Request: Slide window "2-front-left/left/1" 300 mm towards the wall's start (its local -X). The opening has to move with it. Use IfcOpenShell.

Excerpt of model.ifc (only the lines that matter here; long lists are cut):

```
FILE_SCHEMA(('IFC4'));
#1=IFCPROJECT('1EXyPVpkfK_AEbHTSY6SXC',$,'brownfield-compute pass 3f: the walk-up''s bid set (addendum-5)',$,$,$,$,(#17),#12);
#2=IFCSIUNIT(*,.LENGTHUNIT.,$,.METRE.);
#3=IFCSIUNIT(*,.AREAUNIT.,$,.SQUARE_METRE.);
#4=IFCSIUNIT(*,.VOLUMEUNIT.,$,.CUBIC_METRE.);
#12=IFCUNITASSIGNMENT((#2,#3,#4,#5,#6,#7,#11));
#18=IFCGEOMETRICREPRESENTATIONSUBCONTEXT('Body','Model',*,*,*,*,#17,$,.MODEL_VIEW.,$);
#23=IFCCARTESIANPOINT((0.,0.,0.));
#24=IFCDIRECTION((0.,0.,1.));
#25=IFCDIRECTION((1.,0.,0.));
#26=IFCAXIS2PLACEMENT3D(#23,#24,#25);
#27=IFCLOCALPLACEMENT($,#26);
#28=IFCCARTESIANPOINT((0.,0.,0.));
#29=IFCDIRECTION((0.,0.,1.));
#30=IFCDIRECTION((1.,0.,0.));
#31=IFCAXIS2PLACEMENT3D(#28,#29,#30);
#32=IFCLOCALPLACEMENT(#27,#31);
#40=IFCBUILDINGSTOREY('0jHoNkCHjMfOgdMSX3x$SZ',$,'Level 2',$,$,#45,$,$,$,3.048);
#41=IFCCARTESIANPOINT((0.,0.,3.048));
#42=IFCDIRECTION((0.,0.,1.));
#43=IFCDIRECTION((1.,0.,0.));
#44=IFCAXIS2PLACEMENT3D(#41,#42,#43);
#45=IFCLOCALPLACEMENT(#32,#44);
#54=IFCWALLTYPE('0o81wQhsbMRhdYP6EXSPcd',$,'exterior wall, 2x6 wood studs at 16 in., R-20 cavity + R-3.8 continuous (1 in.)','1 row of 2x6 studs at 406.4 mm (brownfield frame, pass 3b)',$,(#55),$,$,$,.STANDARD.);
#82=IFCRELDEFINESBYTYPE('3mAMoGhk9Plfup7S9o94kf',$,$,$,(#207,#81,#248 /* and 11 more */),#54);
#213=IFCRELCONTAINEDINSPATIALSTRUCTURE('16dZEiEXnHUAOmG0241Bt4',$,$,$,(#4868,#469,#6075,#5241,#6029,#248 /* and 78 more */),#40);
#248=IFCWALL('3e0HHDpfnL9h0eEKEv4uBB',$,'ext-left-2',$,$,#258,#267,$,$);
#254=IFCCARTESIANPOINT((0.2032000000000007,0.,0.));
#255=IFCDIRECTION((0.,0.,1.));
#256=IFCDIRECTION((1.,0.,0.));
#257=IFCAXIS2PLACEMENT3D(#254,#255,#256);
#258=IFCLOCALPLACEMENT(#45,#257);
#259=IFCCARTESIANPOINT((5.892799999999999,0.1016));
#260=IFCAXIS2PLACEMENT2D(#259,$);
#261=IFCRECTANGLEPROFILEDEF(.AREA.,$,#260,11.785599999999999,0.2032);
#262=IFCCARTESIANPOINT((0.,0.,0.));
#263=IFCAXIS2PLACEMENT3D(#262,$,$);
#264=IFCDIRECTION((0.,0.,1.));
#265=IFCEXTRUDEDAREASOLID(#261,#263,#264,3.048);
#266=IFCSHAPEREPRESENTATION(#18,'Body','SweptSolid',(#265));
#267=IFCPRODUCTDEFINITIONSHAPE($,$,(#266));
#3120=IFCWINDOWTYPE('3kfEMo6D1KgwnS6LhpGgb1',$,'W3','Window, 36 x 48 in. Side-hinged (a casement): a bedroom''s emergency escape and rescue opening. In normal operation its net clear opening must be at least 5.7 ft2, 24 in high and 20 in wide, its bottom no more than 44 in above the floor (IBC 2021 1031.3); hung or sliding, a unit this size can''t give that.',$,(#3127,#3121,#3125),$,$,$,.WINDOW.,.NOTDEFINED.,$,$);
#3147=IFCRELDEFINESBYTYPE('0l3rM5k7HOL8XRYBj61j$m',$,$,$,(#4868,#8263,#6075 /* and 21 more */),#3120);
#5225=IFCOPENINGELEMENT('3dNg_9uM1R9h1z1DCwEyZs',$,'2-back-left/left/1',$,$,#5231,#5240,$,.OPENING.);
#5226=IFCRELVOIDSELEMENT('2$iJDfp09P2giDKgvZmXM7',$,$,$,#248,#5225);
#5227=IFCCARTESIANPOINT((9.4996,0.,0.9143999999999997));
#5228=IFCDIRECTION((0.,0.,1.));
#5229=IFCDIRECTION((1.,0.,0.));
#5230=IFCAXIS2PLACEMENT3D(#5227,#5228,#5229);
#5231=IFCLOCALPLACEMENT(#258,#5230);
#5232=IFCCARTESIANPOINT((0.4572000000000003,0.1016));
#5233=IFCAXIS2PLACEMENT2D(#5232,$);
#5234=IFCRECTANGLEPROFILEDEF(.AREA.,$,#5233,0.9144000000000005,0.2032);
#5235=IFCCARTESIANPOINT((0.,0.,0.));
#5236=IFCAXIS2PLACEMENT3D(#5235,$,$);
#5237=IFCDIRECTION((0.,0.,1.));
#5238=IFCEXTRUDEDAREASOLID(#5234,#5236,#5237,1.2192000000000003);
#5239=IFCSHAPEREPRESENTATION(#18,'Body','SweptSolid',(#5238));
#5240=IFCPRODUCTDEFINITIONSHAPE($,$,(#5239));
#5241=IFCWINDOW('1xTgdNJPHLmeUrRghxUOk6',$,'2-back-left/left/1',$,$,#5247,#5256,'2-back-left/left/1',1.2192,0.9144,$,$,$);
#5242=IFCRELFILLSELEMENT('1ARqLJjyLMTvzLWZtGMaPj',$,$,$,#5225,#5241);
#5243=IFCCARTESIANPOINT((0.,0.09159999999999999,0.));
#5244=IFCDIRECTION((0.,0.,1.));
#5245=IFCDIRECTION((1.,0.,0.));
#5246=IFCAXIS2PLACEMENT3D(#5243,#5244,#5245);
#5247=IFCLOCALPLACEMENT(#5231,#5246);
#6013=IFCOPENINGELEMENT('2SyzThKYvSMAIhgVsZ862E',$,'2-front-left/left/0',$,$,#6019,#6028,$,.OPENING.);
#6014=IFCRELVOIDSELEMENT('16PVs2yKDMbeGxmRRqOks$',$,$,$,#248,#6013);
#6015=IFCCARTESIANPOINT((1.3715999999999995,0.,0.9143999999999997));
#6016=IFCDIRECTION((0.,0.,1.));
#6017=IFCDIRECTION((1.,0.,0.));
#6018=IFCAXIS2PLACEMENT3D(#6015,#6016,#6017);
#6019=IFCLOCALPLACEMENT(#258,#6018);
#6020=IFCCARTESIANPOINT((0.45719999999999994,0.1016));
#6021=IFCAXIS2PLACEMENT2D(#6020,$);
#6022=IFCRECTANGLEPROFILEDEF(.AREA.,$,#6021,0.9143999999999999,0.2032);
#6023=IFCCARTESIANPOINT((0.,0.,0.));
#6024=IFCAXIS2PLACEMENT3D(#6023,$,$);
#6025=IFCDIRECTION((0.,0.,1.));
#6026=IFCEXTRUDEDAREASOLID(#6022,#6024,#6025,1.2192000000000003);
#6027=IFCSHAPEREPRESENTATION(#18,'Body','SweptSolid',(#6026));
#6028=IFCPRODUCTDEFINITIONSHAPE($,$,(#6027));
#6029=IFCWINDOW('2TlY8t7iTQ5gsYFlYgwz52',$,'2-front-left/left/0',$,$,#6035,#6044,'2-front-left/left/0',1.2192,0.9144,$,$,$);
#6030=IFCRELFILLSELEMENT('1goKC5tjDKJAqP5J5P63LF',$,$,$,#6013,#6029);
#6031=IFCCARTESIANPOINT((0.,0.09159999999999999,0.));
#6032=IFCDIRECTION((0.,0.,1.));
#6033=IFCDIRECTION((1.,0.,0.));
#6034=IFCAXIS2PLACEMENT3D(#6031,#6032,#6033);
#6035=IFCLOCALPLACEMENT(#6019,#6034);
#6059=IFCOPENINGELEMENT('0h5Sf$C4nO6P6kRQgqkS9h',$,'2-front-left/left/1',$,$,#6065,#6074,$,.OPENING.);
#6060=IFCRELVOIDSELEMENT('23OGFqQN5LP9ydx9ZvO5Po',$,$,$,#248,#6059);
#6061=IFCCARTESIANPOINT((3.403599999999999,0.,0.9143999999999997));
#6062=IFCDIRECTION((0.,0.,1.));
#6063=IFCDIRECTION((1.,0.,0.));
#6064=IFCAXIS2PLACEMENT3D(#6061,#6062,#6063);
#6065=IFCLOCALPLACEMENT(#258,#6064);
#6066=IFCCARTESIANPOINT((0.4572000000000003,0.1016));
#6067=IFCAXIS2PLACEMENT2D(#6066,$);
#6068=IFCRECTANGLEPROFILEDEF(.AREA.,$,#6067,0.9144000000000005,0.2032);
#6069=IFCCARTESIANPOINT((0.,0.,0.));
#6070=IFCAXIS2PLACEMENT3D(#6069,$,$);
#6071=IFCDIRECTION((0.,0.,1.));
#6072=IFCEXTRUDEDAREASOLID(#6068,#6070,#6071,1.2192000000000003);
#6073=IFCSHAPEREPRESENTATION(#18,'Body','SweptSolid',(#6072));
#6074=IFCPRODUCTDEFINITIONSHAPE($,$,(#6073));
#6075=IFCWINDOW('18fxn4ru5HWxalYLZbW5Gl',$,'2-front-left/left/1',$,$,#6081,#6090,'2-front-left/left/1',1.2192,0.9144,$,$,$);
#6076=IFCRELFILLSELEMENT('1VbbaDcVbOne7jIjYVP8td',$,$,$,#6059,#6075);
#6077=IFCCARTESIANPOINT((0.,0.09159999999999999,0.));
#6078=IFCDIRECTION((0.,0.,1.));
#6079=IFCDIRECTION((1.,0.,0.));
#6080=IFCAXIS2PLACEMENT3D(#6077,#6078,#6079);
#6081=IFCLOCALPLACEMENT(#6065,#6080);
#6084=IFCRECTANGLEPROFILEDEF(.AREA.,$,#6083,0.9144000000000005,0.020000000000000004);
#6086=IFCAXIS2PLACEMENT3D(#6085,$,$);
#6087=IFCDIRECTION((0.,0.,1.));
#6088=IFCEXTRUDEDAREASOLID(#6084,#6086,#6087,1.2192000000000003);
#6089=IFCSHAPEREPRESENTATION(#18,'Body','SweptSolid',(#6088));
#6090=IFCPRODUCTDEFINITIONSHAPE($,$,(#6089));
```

```python
import ifcopenshell
import ifcopenshell.api.geometry
import ifcopenshell.util.placement
import ifcopenshell.util.unit

model = ifcopenshell.open("model.ifc")
unit_scale = ifcopenshell.util.unit.calculate_unit_scale(model)

window = model.by_guid("18fxn4ru5HWxalYLZbW5Gl")
opening = window.FillsVoids[0].RelatingOpeningElement
wall = opening.VoidsElements[0].RelatingBuildingElement

wall_matrix = ifcopenshell.util.placement.get_local_placement(wall.ObjectPlacement)
shift = wall_matrix[:3, 0] * -0.3 / unit_scale
before = ifcopenshell.util.placement.get_local_placement(window.ObjectPlacement)[:3, 3].copy()

# The window is placed relative to its opening, so it follows when the opening moves.
matrix = ifcopenshell.util.placement.get_local_placement(opening.ObjectPlacement)
matrix[:3, 3] += shift
ifcopenshell.api.geometry.edit_object_placement(
    model, product=opening, matrix=matrix, is_si=False, should_transform_children=True
)

after = ifcopenshell.util.placement.get_local_placement(window.ObjectPlacement)[:3, 3]
print("window moved by", (after - before).round(3) + 0.0)

model.write("model_rev.ifc")
```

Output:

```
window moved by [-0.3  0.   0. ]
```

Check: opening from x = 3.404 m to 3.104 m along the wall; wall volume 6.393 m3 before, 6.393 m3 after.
